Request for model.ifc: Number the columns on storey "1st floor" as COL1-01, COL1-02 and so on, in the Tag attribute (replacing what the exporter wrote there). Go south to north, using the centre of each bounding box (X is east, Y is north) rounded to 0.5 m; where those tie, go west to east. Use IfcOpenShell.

First a look at what the model holds.

```python
import ifcopenshell
import ifcopenshell.util.element
import ifcopenshell.util.placement

model = ifcopenshell.open("model.ifc")
print(model.schema)
storey = next(s for s in model.by_type("IfcBuildingStorey") if s.Name == "1st floor")
columns = [e for e in ifcopenshell.util.element.get_decomposition(storey) if e.is_a("IfcColumn")]
for e in sorted(columns, key=lambda e: e.id()):
    origin = ifcopenshell.util.placement.get_local_placement(e.ObjectPlacement)[:3, 3]
    print(e.id(), e.Tag, e.Name, origin.round(2) + 0.0, sep=" | ")
```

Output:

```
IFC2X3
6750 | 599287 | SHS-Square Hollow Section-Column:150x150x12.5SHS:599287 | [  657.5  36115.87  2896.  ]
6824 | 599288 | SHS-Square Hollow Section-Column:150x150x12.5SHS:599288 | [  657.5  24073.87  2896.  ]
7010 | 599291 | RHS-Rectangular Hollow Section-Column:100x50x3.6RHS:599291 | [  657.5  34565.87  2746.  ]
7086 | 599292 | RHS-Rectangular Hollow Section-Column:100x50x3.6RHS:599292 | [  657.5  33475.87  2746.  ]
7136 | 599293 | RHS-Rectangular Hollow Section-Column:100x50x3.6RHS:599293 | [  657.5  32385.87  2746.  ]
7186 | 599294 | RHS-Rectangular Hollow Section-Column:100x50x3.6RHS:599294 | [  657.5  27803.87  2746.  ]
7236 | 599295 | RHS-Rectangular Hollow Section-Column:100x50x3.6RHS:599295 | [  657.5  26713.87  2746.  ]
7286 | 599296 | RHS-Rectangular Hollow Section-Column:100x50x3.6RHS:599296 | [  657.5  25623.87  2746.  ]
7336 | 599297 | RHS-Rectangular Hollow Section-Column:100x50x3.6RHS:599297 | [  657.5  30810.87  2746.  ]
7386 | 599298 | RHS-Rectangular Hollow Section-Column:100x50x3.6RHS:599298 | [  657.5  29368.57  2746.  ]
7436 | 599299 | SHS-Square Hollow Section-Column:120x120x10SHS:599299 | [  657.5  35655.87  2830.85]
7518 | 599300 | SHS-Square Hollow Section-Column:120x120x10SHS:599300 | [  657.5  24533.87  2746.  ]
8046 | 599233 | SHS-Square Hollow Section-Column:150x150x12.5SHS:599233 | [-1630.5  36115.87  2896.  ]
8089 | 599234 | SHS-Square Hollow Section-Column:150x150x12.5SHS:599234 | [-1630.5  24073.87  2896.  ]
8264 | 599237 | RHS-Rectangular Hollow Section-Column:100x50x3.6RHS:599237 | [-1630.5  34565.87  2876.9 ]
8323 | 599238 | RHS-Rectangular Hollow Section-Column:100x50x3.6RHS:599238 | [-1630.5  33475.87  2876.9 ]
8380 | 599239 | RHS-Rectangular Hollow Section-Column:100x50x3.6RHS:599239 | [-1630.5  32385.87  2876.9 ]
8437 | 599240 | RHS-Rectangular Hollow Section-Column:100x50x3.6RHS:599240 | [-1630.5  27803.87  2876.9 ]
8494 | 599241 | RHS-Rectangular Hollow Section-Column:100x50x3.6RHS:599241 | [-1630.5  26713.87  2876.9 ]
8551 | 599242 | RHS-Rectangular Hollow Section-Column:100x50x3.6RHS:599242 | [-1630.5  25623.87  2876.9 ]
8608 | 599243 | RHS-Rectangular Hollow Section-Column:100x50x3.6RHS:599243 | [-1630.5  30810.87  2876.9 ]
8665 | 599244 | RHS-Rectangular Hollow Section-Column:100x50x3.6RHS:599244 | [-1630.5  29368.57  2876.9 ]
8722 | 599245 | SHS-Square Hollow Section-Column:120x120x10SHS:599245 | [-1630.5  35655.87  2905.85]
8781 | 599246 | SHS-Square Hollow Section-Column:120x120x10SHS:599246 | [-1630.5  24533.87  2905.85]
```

```python
import ifcopenshell
import ifcopenshell.geom
import ifcopenshell.util.element
import ifcopenshell.util.shape

model = ifcopenshell.open("model.ifc")
settings = ifcopenshell.geom.settings()
settings.set("use-world-coords", True)


def centre(element):
    shape = ifcopenshell.geom.create_shape(settings, element)
    return ifcopenshell.util.shape.get_bbox_centroid(shape.geometry)


storey = next(s for s in model.by_type("IfcBuildingStorey") if s.Name == "1st floor")
columns = [e for e in ifcopenshell.util.element.get_decomposition(storey) if e.is_a("IfcColumn")]

# Insertion points can sit at a corner or the storey origin, so sort by the geometry (in metres).
centres = {e: centre(e) for e in columns}
columns.sort(key=lambda e: (round(centres[e][1] / 0.5), centres[e][0]))

for i, e in enumerate(columns, start=1):
    number = f"COL1-{i:02d}"
    e.Tag = number
    print(e.id(), number)

model.write("model_edited.ifc")
```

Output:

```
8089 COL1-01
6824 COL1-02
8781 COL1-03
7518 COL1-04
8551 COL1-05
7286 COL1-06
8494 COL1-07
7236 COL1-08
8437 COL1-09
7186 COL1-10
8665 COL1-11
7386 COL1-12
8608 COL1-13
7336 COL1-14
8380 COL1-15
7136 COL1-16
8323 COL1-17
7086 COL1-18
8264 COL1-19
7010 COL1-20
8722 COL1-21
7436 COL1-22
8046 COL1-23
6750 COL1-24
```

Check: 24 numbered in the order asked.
